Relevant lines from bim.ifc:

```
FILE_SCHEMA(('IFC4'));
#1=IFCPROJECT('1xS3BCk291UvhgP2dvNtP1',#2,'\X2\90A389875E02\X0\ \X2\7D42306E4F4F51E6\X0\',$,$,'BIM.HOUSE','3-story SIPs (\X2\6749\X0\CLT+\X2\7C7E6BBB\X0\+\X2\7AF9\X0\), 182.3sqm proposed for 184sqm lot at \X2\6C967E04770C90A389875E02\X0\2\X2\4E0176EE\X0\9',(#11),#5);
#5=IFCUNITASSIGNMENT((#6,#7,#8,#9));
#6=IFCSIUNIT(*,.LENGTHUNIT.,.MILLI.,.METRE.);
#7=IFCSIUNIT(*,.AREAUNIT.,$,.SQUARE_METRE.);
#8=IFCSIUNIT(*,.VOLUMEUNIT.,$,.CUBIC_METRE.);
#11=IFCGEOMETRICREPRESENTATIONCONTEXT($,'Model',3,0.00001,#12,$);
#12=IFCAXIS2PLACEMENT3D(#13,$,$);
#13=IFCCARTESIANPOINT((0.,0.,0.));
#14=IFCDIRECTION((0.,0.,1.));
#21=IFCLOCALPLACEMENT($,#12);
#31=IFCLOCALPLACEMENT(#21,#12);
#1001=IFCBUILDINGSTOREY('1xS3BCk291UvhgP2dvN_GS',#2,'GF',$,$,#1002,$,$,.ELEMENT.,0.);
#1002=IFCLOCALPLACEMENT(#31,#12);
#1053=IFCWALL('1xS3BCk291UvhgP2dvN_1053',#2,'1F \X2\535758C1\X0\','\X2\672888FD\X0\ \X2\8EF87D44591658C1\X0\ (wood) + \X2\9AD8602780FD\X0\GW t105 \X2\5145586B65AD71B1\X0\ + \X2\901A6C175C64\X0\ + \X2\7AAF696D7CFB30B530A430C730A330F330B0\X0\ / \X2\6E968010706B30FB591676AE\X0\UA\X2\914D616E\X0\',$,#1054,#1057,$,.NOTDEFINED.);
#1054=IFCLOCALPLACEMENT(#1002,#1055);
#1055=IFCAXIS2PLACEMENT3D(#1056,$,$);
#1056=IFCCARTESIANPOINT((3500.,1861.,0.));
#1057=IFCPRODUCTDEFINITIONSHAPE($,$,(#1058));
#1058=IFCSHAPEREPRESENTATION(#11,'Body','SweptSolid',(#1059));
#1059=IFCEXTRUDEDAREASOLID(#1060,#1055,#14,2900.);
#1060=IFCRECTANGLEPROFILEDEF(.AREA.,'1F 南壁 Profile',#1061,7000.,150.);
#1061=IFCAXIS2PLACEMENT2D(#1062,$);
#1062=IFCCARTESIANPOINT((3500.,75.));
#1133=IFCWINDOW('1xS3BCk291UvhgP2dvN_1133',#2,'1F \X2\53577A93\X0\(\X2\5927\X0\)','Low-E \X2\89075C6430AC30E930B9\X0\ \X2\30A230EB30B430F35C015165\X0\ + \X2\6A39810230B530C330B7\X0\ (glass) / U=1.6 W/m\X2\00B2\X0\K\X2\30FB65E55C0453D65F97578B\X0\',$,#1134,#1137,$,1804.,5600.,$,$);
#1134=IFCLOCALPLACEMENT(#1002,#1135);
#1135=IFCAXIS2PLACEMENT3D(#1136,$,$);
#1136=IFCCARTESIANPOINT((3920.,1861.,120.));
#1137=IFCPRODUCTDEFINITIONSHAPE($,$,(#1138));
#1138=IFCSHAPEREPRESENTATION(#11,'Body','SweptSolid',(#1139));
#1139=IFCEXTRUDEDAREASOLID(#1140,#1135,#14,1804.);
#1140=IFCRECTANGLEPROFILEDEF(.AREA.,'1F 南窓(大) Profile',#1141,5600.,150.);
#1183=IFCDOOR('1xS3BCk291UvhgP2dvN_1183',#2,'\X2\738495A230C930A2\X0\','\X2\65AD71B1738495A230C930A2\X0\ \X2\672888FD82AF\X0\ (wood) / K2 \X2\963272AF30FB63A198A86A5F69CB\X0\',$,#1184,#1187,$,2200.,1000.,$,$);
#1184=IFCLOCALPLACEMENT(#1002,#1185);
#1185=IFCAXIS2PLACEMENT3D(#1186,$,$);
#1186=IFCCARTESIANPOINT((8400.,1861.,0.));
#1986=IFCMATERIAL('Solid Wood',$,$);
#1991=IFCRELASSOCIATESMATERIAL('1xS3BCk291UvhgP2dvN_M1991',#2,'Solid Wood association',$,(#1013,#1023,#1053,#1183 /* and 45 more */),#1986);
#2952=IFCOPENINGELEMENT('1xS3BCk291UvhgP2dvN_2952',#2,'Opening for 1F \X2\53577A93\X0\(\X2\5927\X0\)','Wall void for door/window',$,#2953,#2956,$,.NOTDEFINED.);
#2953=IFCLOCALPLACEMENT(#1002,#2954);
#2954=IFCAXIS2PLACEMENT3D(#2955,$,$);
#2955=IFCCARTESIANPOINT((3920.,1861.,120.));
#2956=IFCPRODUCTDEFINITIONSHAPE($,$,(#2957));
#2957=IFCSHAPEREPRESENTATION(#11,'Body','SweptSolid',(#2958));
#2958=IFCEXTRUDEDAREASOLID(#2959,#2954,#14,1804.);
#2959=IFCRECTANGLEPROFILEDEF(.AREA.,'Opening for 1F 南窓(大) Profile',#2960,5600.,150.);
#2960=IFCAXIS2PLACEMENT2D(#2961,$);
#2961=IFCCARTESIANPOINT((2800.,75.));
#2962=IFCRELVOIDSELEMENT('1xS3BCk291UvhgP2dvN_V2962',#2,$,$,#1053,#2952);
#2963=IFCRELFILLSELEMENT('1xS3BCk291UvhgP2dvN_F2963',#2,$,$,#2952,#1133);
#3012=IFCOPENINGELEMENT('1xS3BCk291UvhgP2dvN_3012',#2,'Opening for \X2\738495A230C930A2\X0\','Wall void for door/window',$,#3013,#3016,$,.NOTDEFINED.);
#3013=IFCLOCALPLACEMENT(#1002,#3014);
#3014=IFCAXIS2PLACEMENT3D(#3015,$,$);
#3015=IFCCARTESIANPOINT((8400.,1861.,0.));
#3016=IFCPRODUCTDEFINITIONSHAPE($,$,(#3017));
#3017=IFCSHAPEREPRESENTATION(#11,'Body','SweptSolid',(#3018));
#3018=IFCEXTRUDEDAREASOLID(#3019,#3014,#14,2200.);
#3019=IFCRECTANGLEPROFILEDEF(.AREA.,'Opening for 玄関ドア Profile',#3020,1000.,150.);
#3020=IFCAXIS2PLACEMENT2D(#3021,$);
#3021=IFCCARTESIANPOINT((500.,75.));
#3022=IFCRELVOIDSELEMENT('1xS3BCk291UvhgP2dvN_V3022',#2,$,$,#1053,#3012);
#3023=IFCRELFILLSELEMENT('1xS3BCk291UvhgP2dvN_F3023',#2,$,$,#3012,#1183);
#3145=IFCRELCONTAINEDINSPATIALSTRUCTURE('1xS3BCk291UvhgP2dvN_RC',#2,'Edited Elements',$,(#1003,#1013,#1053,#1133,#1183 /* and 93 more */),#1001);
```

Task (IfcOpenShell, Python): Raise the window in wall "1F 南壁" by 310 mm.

```python
import numpy as np
import ifcopenshell
import ifcopenshell.api.geometry
import ifcopenshell.util.placement
import ifcopenshell.util.unit

model = ifcopenshell.open("bim.ifc")
unit_scale = ifcopenshell.util.unit.calculate_unit_scale(model)

window = model.by_guid("1xS3BCk291UvhgP2dvN_1133")
opening = window.FillsVoids[0].RelatingOpeningElement
dz = 0.31 / unit_scale

shift = np.array([0.0, 0.0, dz])
# The window is not placed relative to its opening, so move both.
for product in (opening, window):
    matrix = ifcopenshell.util.placement.get_local_placement(product.ObjectPlacement)
    matrix[:3, 3] += shift
    ifcopenshell.api.geometry.edit_object_placement(model, product=product, matrix=matrix, is_si=False)

print(f"moved by {dz * unit_scale:+.3f} m")

model.write("bim_updated.ifc")
```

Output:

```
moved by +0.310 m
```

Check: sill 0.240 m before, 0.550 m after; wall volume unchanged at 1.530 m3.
